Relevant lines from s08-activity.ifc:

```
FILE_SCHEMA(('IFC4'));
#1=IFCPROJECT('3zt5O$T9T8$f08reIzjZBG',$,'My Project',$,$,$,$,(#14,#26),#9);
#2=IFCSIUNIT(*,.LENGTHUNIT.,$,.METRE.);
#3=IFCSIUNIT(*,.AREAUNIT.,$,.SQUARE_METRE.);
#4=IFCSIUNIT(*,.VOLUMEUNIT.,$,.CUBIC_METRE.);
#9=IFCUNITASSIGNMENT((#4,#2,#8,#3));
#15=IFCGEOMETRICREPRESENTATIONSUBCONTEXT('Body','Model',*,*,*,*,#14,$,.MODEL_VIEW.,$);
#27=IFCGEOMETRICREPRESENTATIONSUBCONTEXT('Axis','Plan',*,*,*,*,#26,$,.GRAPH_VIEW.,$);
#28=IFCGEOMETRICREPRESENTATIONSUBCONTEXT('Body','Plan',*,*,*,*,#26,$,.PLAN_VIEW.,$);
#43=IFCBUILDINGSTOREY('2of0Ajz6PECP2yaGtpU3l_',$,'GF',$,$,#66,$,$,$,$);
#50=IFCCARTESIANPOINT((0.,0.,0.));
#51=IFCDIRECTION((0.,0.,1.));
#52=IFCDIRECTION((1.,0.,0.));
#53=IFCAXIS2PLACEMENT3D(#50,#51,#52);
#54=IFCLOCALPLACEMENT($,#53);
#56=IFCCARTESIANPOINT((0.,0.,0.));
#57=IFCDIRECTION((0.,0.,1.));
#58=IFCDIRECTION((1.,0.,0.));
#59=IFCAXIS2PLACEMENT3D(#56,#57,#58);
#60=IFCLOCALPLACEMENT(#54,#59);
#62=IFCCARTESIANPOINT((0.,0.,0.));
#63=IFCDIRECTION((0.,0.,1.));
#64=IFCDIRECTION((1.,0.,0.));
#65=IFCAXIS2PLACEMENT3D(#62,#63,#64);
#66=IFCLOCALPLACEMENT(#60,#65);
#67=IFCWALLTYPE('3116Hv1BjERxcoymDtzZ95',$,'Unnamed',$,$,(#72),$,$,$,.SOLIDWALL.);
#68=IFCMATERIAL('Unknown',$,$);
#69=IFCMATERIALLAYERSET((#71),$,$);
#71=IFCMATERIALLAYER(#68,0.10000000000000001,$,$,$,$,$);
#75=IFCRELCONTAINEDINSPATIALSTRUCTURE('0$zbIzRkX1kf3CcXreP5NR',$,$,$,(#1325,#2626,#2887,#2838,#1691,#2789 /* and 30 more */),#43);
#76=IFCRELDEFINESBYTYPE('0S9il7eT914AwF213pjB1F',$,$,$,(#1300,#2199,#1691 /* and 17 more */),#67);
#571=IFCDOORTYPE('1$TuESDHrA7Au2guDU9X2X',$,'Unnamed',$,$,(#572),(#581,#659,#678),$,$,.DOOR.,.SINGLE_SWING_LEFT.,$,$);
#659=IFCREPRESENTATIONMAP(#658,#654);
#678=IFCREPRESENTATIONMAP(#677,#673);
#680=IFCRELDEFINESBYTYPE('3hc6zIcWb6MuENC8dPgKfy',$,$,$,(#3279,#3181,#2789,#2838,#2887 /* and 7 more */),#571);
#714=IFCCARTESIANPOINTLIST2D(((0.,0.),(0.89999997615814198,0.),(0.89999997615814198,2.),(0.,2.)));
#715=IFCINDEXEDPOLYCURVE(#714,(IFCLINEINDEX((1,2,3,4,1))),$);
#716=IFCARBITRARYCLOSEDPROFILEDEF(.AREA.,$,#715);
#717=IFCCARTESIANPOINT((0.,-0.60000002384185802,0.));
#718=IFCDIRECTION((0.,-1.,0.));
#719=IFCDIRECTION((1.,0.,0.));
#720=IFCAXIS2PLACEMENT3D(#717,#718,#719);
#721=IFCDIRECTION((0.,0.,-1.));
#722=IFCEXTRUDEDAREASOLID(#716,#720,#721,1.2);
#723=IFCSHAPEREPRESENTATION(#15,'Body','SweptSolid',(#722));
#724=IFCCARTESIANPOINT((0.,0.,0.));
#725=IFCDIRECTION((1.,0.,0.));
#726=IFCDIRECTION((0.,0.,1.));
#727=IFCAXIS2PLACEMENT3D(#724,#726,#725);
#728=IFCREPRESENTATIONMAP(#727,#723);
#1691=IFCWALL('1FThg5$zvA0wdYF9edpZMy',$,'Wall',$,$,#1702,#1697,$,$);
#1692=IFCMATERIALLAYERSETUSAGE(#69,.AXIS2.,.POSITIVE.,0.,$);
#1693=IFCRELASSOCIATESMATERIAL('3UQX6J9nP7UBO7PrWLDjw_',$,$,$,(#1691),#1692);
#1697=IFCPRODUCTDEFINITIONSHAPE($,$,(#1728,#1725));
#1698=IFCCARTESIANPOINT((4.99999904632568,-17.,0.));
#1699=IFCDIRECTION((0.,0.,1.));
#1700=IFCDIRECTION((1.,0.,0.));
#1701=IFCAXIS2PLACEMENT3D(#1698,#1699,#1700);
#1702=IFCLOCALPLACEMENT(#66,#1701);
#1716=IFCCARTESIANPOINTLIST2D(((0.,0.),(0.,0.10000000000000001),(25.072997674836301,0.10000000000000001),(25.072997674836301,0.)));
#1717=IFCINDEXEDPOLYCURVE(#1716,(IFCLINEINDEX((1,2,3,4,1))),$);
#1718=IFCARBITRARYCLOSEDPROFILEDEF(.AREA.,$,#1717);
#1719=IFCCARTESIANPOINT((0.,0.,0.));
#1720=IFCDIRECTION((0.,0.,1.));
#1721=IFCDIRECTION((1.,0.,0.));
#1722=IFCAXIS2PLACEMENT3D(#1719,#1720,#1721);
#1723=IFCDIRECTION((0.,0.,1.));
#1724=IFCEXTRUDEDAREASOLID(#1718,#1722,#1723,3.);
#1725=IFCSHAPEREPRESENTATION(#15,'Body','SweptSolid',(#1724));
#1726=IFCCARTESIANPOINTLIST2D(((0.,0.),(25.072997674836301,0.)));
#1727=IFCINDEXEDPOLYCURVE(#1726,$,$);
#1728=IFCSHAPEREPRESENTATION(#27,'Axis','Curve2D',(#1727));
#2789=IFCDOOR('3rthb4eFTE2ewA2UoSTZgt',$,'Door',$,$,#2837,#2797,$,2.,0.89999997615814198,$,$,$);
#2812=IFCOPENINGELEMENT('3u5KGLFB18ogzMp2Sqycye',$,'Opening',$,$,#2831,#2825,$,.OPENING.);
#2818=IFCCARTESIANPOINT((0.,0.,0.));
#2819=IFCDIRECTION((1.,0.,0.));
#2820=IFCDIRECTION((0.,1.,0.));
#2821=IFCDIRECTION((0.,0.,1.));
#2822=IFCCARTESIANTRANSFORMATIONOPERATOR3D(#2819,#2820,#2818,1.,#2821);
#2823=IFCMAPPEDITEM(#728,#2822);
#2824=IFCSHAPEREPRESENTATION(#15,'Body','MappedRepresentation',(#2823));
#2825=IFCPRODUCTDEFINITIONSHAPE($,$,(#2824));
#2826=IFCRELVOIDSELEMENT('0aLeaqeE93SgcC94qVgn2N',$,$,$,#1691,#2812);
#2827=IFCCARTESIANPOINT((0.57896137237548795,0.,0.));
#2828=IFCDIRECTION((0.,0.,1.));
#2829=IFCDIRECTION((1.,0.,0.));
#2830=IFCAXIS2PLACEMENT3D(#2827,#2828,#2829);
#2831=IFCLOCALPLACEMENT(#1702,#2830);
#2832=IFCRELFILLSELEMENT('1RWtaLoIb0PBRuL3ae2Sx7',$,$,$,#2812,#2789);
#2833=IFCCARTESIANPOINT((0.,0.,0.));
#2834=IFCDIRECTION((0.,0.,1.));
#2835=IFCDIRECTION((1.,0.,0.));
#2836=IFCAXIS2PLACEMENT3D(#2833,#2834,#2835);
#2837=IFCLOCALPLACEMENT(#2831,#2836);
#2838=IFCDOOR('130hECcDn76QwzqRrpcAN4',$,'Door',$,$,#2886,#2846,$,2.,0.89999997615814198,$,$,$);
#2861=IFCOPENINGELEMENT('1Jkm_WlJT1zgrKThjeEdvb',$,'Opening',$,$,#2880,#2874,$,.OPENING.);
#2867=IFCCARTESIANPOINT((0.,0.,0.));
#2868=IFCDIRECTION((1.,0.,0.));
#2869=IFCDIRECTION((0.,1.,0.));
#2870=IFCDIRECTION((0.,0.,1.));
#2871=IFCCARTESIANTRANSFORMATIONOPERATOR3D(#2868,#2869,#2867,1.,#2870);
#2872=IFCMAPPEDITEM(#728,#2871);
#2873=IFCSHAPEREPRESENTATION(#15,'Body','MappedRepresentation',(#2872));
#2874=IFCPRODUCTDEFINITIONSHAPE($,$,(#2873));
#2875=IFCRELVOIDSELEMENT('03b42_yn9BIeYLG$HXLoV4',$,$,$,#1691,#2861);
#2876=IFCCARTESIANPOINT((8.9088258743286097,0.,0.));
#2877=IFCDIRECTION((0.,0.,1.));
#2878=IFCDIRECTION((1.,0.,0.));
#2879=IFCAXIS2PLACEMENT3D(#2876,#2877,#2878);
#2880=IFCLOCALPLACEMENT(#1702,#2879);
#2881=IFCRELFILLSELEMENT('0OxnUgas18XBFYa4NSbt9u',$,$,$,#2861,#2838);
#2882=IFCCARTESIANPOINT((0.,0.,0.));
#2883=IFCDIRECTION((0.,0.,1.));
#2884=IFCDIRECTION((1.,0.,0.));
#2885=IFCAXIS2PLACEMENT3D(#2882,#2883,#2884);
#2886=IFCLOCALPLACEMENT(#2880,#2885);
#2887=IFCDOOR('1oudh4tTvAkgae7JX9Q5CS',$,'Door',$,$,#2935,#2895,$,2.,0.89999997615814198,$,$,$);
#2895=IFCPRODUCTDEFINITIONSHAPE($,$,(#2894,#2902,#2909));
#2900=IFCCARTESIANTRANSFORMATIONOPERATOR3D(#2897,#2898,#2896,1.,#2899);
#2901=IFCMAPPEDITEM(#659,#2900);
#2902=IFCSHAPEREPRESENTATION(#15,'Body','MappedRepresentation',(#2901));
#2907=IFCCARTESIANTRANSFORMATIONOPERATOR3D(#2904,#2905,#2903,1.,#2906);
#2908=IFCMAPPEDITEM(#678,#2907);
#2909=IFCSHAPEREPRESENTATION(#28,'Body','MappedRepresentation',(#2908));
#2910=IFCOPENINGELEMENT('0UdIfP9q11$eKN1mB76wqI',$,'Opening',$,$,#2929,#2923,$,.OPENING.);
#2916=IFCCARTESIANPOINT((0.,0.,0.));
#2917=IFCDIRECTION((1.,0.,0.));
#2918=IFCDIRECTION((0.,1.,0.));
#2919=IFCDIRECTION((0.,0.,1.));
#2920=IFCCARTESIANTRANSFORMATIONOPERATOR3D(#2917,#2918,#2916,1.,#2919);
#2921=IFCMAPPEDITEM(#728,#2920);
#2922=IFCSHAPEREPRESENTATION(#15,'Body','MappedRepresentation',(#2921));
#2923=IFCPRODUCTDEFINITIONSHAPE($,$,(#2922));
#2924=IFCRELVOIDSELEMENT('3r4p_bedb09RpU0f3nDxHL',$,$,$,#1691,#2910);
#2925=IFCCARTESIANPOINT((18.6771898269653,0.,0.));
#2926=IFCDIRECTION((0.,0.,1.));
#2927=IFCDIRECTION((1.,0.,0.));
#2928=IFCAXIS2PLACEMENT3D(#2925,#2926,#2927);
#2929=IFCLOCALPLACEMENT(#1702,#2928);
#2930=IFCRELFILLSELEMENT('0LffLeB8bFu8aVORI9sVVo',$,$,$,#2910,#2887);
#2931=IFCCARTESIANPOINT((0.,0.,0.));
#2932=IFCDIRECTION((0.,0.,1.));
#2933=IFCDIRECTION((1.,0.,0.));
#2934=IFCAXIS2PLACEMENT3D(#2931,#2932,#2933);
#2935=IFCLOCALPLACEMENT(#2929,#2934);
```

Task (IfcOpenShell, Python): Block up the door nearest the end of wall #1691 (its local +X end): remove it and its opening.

```python
import ifcopenshell
import ifcopenshell.api.feature
import ifcopenshell.api.root
import ifcopenshell.geom
import ifcopenshell.util.shape

model = ifcopenshell.open("s08-activity.ifc")
settings = ifcopenshell.geom.settings()


def volume(element):
    """Net volume in cubic metres, openings subtracted."""
    shape = ifcopenshell.geom.create_shape(settings, element)
    return ifcopenshell.util.shape.get_volume(shape.geometry)


door = model.by_guid("1oudh4tTvAkgae7JX9Q5CS")
opening = door.FillsVoids[0].RelatingOpeningElement
wall = opening.VoidsElements[0].RelatingBuildingElement
before = volume(wall)

ifcopenshell.api.root.remove_product(model, product=door)
ifcopenshell.api.feature.remove_feature(model, feature=opening)

after = volume(wall)

print(f"wall volume {before:.3f} -> {after:.3f} m3")

model.write("s08-activity-out.ifc")
```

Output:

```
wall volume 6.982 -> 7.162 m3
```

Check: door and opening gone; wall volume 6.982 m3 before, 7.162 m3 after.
